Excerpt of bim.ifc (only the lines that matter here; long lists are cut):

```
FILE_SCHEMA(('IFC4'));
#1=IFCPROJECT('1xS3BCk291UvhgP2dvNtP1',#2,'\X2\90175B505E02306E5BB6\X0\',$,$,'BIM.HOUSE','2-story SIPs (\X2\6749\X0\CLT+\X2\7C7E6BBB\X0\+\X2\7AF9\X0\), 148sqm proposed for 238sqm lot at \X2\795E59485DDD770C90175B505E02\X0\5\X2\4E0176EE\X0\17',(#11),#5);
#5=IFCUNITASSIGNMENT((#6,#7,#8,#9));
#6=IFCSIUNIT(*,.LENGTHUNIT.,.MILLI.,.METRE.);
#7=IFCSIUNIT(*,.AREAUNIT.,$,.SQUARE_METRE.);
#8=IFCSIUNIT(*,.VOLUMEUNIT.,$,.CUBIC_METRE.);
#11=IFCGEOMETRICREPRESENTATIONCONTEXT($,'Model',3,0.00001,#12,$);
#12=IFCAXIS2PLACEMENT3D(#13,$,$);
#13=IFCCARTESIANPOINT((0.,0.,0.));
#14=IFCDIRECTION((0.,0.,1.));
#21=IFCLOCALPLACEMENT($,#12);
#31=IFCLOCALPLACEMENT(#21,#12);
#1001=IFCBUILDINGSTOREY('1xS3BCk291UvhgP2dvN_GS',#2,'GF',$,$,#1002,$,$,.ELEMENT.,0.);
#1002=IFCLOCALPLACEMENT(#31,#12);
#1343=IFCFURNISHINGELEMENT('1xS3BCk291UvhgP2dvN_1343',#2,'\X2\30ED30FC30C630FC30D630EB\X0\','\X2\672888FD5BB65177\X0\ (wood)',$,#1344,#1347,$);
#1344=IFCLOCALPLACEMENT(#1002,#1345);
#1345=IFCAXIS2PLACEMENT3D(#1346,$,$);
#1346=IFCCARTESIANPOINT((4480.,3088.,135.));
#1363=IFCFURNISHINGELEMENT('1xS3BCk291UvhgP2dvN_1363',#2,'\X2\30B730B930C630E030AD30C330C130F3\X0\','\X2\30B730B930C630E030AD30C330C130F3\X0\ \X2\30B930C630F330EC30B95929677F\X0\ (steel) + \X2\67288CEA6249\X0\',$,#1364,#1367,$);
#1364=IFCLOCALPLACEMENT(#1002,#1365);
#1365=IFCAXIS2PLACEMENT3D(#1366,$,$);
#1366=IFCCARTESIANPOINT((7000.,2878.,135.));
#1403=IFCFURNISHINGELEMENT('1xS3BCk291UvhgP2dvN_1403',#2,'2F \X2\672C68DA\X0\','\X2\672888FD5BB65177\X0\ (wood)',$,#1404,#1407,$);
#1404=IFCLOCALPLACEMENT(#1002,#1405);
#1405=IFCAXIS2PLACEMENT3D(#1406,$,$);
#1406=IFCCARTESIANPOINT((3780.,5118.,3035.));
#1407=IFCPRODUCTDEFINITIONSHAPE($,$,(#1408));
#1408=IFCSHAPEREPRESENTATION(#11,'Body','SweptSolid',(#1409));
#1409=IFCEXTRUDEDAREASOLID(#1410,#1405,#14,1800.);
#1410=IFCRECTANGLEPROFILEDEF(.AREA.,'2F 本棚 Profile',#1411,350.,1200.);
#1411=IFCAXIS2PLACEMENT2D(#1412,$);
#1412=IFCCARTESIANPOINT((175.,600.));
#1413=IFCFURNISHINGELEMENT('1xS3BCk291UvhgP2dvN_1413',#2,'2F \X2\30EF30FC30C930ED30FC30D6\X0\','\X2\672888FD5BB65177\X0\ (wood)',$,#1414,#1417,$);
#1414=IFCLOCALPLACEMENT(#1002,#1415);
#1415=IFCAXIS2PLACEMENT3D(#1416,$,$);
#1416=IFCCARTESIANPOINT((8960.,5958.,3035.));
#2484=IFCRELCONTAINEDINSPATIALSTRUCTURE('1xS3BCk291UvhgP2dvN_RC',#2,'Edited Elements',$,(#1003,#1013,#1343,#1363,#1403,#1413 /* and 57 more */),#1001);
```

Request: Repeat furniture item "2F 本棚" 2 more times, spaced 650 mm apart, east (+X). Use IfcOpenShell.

```python
import numpy as np
import ifcopenshell
import ifcopenshell.api.geometry
import ifcopenshell.api.root
import ifcopenshell.util.element
import ifcopenshell.util.placement

model = ifcopenshell.open("bim.ifc")


def reuse_history(source, copy):
    """copy_class also copies each property set's owner history, people and application; keep the originals."""
    for rel in copy.IsDefinedBy:
        if rel.is_a("IfcRelDefinesByProperties") and (history := rel.RelatingPropertyDefinition.OwnerHistory):
            rel.RelatingPropertyDefinition.OwnerHistory = source.OwnerHistory
            ifcopenshell.util.element.remove_deep2(model, history)


source = model.by_guid("1xS3BCk291UvhgP2dvN_1403")
base = ifcopenshell.util.placement.get_local_placement(source.ObjectPlacement)
step = np.array([1.0, 0.0, 0.0]) * 650.0

for i in range(1, 3):
    copy = ifcopenshell.api.root.copy_class(model, product=source)
    copy.Representation = ifcopenshell.util.element.copy_deep(
        model, source.Representation, exclude=["IfcGeometricRepresentationContext", "IfcRepresentationMap"]
    )
    reuse_history(source, copy)
    matrix = base.copy()
    matrix[:3, 3] += i * step
    print("added at", matrix[:3, 3].round(3) + 0.0)
    ifcopenshell.api.geometry.edit_object_placement(model, product=copy, matrix=matrix, is_si=False)

model.write("bim-out.ifc")
```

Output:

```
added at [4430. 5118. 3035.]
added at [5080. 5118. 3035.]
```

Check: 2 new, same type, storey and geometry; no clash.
